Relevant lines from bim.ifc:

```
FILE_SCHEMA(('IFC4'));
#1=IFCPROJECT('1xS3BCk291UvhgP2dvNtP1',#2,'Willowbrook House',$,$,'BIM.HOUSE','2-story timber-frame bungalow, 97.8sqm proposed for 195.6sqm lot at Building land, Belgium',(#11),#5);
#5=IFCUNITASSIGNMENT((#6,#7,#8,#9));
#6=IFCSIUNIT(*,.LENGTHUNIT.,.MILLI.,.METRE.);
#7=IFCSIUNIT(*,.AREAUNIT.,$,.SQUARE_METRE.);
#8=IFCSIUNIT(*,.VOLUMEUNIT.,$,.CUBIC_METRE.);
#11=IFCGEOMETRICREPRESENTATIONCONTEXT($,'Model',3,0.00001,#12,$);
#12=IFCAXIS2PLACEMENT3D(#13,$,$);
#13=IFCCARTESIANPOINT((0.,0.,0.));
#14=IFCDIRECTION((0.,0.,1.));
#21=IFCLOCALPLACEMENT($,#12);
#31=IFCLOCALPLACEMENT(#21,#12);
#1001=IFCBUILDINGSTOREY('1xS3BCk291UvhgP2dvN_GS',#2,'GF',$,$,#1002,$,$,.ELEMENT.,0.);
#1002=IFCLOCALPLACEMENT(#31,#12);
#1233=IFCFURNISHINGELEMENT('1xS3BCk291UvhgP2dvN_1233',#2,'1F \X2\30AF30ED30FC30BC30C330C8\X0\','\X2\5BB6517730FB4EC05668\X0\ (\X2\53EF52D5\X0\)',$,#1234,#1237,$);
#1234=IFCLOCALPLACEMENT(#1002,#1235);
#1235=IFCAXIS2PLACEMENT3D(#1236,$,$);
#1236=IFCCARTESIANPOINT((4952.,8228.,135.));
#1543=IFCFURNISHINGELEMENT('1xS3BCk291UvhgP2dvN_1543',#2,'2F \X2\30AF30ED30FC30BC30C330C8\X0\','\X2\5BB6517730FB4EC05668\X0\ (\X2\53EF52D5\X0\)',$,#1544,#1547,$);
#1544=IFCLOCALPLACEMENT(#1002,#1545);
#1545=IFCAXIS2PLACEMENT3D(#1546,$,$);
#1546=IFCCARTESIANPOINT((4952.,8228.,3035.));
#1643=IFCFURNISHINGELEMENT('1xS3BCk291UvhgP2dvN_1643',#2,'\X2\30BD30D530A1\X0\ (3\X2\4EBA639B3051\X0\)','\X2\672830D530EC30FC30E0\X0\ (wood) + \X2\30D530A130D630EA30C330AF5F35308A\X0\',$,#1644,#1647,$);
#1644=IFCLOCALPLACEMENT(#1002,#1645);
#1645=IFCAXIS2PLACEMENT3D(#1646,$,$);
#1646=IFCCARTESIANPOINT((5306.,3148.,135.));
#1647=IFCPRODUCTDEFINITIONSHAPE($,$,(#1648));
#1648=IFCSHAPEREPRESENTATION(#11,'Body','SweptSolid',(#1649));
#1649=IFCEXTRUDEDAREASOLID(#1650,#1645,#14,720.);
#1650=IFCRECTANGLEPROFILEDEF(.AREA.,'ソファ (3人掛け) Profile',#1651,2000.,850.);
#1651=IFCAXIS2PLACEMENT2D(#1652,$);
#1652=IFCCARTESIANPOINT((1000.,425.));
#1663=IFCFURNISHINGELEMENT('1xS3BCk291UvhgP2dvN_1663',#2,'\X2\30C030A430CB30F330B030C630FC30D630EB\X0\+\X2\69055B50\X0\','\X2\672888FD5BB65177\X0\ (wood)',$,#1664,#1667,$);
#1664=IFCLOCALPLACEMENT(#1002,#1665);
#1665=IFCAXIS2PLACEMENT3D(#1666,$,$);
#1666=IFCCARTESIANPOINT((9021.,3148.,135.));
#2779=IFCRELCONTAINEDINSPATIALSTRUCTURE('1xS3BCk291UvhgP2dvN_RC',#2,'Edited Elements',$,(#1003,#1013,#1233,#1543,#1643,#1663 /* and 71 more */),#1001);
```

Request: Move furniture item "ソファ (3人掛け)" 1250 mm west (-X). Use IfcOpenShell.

```python
import ifcopenshell
import ifcopenshell.api.geometry
import ifcopenshell.util.placement
import ifcopenshell.util.unit

model = ifcopenshell.open("bim.ifc")
unit_scale = ifcopenshell.util.unit.calculate_unit_scale(model)

item = model.by_guid("1xS3BCk291UvhgP2dvN_1643")
matrix = ifcopenshell.util.placement.get_local_placement(item.ObjectPlacement)
matrix[0, 3] -= 1.25 / unit_scale
ifcopenshell.api.geometry.edit_object_placement(model, product=item, matrix=matrix, is_si=False)

print(ifcopenshell.util.placement.get_local_placement(item.ObjectPlacement).round(3) + 0.0)

model.write("bim_edited.ifc")
```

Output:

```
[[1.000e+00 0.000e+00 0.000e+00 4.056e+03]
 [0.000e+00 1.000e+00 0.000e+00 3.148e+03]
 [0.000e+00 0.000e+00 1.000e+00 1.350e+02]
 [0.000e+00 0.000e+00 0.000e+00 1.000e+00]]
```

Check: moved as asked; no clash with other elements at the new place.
